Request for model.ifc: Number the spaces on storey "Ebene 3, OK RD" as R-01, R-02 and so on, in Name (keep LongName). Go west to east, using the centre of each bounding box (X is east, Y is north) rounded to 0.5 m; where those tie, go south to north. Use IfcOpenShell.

First a look at what the model holds.

```python
import ifcopenshell
import ifcopenshell.util.element
import ifcopenshell.util.placement

model = ifcopenshell.open("model.ifc")
print(model.schema)
storey = next(s for s in model.by_type("IfcBuildingStorey") if s.Name == "Ebene 3, OK RD")
spaces = [e for e in ifcopenshell.util.element.get_decomposition(storey) if e.is_a("IfcSpace")]
for e in sorted(spaces, key=lambda e: e.id()):
    origin = ifcopenshell.util.placement.get_local_placement(e.ObjectPlacement)[:3, 3]
    print(e.id(), e.Name, e.LongName, origin.round(2) + 0.0, sep=" | ")
```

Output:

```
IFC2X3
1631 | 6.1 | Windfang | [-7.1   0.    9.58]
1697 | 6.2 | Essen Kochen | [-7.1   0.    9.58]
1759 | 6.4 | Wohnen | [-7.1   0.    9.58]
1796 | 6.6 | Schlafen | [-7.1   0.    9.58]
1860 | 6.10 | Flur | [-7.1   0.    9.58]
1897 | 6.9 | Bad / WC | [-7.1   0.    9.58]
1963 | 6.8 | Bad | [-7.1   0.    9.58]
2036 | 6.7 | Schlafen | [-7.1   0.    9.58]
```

```python
import ifcopenshell
import ifcopenshell.geom
import ifcopenshell.util.element
import ifcopenshell.util.shape

model = ifcopenshell.open("model.ifc")
settings = ifcopenshell.geom.settings()
settings.set("use-world-coords", True)


def centre(element):
    shape = ifcopenshell.geom.create_shape(settings, element)
    return ifcopenshell.util.shape.get_bbox_centroid(shape.geometry)


storey = next(s for s in model.by_type("IfcBuildingStorey") if s.Name == "Ebene 3, OK RD")
spaces = [e for e in ifcopenshell.util.element.get_decomposition(storey) if e.is_a("IfcSpace")]

# Insertion points can sit at a corner or the storey origin, so sort by the geometry (in metres).
centres = {e: centre(e) for e in spaces}
spaces.sort(key=lambda e: (round(centres[e][0] / 0.5), centres[e][1]))

for i, e in enumerate(spaces, start=1):
    number = f"R-{i:02d}"
    e.Name = number
    print(e.id(), number)

model.write("model_updated.ifc")
```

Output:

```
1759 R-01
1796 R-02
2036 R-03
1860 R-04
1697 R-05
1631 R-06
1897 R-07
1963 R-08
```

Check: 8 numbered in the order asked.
